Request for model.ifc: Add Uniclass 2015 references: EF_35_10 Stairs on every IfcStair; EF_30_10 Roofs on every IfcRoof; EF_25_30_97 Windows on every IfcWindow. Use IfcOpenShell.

First a look at what the model holds.

```python
import ifcopenshell

model = ifcopenshell.open("model.ifc")
print(model.schema)
print("classifications:", [c.Name for c in model.by_type("IfcClassification")])
for ifc_class in ("IfcDoor", "IfcRoof", "IfcStair", "IfcWall", "IfcWindow"):
    print(ifc_class, len(model.by_type(ifc_class)))
```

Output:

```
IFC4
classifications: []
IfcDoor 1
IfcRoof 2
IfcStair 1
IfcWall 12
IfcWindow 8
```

```python
import ifcopenshell
import ifcopenshell.api.classification

model = ifcopenshell.open("model.ifc")

system = ifcopenshell.api.classification.add_classification(model, classification="Uniclass 2015")

codes = {
    "IfcStair": ("EF_35_10", "Stairs"),
    "IfcRoof": ("EF_30_10", "Roofs"),
    "IfcWindow": ("EF_25_30_97", "Windows"),
}
for ifc_class, (code, name) in codes.items():
    products = model.by_type(ifc_class)
    ifcopenshell.api.classification.add_reference(
        model, products=products, classification=system, identification=code, name=name
    )
    print(code, len(products))

model.write("model_rev.ifc")
```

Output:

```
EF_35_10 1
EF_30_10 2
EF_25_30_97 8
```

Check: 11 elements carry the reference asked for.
